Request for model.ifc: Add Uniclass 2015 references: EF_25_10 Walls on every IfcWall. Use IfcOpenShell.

First a look at what the model holds.

```python
import ifcopenshell

model = ifcopenshell.open("model.ifc")
print(model.schema)
print("classifications:", [c.Name for c in model.by_type("IfcClassification")])
for ifc_class in ("IfcDoor", "IfcRoof", "IfcStair", "IfcWall", "IfcWindow"):
    print(ifc_class, len(model.by_type(ifc_class)))
```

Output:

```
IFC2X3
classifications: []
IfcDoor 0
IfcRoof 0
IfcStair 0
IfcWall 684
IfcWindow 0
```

```python
import ifcopenshell
import ifcopenshell.api.classification

model = ifcopenshell.open("model.ifc")

# IFC2X3 requires Source and Edition and has no link from the project to the system.
system = model.create_entity("IfcClassification", Source="NBS", Edition="2015", Name="Uniclass 2015")

codes = {
    "IfcWall": ("EF_25_10", "Walls"),
}
for ifc_class, (code, name) in codes.items():
    products = model.by_type(ifc_class)
    ifcopenshell.api.classification.add_reference(
        model, products=products, classification=system, identification=code, name=name
    )
    print(code, len(products))

model.write("model_updated.ifc")
```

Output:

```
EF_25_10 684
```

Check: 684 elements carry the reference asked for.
